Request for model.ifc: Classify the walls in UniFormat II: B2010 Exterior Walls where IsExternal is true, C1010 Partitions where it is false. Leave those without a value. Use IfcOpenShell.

First a look at what the model holds.

```python
import ifcopenshell
import ifcopenshell.util.element

model = ifcopenshell.open("model.ifc")
print(model.schema)
print("classifications:", [c.Name for c in model.by_type("IfcClassification")])
values = [ifcopenshell.util.element.get_pset(e, "Pset_WallCommon", "IsExternal") for e in model.by_type("IfcWall")]
for value in (True, False, None):
    print("IsExternal", value, values.count(value))
```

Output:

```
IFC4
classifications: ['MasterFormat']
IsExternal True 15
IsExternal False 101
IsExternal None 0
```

```python
import ifcopenshell
import ifcopenshell.api.classification
import ifcopenshell.util.element

model = ifcopenshell.open("model.ifc")

system = ifcopenshell.api.classification.add_classification(model, classification="UniFormat II")

walls = model.by_type("IfcWall")
external = {e: ifcopenshell.util.element.get_pset(e, "Pset_WallCommon", "IsExternal") for e in walls}
for flag, code, name in ((True, "B2010", "Exterior Walls"), (False, "C1010", "Partitions")):
    products = [e for e in walls if external[e] is flag]
    ifcopenshell.api.classification.add_reference(
        model, products=products, classification=system, identification=code, name=name
    )
    print(code, len(products))

model.write("model_v2.ifc")
```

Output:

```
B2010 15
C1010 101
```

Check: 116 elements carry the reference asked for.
